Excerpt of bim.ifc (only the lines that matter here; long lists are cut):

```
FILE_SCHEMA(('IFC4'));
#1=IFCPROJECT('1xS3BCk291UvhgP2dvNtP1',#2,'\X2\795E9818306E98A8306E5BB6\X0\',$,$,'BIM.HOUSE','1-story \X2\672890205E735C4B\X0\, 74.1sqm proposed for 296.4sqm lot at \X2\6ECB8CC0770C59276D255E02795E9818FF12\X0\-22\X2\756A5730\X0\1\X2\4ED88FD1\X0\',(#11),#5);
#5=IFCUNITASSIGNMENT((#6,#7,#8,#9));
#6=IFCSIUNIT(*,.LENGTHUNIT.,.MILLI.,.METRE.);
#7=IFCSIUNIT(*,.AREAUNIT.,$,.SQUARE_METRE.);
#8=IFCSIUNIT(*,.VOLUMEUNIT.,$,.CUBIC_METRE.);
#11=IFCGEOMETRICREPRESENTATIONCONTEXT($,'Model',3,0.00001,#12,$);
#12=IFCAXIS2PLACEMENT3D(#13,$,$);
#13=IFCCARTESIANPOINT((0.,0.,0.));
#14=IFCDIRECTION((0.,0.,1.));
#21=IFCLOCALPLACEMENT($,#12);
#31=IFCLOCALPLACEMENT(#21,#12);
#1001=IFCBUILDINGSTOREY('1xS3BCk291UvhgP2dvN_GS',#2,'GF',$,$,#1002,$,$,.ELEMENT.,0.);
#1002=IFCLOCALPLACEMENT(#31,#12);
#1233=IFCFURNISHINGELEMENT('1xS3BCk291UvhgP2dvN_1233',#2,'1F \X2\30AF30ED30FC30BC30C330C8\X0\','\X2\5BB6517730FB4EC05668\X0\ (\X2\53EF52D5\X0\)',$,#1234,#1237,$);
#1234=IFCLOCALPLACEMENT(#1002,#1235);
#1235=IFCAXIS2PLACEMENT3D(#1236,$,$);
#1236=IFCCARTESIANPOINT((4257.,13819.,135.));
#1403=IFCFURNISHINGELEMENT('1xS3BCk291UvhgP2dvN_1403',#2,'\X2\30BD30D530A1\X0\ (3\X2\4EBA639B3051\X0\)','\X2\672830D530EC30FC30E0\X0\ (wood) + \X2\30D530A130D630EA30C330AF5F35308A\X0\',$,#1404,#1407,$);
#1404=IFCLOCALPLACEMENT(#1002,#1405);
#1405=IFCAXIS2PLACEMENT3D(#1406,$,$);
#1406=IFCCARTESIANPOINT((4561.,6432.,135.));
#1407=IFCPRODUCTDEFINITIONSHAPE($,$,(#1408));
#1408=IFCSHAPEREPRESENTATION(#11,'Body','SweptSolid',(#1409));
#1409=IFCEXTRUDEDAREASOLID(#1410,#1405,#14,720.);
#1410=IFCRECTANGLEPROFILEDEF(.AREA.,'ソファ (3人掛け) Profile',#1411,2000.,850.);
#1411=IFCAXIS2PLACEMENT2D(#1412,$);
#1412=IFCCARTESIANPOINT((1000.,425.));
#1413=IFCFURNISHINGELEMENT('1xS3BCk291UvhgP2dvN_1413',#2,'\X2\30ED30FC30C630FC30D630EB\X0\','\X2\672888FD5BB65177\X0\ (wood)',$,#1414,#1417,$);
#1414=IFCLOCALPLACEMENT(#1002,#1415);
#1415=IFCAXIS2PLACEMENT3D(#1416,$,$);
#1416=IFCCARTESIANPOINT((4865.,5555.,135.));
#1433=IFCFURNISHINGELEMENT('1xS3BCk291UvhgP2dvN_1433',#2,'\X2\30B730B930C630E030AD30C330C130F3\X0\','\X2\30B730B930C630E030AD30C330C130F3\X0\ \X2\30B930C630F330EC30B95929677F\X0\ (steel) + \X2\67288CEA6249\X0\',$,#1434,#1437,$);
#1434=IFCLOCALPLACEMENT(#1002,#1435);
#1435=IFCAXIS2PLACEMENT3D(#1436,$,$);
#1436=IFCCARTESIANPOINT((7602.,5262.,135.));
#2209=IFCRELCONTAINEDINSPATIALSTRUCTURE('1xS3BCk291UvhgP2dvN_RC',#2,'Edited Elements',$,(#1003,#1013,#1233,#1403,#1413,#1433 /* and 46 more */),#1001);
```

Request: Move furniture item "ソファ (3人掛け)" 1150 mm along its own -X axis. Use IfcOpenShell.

```python
import ifcopenshell
import ifcopenshell.api.geometry
import ifcopenshell.util.placement

model = ifcopenshell.open("bim.ifc")

item = model.by_id(1403)
matrix = ifcopenshell.util.placement.get_local_placement(item.ObjectPlacement)
matrix[:3, 3] -= matrix[:3, 0] * 1150.0
ifcopenshell.api.geometry.edit_object_placement(model, product=item, matrix=matrix, is_si=False)

print(ifcopenshell.util.placement.get_local_placement(item.ObjectPlacement).round(3) + 0.0)

model.write("bim_edited.ifc")
```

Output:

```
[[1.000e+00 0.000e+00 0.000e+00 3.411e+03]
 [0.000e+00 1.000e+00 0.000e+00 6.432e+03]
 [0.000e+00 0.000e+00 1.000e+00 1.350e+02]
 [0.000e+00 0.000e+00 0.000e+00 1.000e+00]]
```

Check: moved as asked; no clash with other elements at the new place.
